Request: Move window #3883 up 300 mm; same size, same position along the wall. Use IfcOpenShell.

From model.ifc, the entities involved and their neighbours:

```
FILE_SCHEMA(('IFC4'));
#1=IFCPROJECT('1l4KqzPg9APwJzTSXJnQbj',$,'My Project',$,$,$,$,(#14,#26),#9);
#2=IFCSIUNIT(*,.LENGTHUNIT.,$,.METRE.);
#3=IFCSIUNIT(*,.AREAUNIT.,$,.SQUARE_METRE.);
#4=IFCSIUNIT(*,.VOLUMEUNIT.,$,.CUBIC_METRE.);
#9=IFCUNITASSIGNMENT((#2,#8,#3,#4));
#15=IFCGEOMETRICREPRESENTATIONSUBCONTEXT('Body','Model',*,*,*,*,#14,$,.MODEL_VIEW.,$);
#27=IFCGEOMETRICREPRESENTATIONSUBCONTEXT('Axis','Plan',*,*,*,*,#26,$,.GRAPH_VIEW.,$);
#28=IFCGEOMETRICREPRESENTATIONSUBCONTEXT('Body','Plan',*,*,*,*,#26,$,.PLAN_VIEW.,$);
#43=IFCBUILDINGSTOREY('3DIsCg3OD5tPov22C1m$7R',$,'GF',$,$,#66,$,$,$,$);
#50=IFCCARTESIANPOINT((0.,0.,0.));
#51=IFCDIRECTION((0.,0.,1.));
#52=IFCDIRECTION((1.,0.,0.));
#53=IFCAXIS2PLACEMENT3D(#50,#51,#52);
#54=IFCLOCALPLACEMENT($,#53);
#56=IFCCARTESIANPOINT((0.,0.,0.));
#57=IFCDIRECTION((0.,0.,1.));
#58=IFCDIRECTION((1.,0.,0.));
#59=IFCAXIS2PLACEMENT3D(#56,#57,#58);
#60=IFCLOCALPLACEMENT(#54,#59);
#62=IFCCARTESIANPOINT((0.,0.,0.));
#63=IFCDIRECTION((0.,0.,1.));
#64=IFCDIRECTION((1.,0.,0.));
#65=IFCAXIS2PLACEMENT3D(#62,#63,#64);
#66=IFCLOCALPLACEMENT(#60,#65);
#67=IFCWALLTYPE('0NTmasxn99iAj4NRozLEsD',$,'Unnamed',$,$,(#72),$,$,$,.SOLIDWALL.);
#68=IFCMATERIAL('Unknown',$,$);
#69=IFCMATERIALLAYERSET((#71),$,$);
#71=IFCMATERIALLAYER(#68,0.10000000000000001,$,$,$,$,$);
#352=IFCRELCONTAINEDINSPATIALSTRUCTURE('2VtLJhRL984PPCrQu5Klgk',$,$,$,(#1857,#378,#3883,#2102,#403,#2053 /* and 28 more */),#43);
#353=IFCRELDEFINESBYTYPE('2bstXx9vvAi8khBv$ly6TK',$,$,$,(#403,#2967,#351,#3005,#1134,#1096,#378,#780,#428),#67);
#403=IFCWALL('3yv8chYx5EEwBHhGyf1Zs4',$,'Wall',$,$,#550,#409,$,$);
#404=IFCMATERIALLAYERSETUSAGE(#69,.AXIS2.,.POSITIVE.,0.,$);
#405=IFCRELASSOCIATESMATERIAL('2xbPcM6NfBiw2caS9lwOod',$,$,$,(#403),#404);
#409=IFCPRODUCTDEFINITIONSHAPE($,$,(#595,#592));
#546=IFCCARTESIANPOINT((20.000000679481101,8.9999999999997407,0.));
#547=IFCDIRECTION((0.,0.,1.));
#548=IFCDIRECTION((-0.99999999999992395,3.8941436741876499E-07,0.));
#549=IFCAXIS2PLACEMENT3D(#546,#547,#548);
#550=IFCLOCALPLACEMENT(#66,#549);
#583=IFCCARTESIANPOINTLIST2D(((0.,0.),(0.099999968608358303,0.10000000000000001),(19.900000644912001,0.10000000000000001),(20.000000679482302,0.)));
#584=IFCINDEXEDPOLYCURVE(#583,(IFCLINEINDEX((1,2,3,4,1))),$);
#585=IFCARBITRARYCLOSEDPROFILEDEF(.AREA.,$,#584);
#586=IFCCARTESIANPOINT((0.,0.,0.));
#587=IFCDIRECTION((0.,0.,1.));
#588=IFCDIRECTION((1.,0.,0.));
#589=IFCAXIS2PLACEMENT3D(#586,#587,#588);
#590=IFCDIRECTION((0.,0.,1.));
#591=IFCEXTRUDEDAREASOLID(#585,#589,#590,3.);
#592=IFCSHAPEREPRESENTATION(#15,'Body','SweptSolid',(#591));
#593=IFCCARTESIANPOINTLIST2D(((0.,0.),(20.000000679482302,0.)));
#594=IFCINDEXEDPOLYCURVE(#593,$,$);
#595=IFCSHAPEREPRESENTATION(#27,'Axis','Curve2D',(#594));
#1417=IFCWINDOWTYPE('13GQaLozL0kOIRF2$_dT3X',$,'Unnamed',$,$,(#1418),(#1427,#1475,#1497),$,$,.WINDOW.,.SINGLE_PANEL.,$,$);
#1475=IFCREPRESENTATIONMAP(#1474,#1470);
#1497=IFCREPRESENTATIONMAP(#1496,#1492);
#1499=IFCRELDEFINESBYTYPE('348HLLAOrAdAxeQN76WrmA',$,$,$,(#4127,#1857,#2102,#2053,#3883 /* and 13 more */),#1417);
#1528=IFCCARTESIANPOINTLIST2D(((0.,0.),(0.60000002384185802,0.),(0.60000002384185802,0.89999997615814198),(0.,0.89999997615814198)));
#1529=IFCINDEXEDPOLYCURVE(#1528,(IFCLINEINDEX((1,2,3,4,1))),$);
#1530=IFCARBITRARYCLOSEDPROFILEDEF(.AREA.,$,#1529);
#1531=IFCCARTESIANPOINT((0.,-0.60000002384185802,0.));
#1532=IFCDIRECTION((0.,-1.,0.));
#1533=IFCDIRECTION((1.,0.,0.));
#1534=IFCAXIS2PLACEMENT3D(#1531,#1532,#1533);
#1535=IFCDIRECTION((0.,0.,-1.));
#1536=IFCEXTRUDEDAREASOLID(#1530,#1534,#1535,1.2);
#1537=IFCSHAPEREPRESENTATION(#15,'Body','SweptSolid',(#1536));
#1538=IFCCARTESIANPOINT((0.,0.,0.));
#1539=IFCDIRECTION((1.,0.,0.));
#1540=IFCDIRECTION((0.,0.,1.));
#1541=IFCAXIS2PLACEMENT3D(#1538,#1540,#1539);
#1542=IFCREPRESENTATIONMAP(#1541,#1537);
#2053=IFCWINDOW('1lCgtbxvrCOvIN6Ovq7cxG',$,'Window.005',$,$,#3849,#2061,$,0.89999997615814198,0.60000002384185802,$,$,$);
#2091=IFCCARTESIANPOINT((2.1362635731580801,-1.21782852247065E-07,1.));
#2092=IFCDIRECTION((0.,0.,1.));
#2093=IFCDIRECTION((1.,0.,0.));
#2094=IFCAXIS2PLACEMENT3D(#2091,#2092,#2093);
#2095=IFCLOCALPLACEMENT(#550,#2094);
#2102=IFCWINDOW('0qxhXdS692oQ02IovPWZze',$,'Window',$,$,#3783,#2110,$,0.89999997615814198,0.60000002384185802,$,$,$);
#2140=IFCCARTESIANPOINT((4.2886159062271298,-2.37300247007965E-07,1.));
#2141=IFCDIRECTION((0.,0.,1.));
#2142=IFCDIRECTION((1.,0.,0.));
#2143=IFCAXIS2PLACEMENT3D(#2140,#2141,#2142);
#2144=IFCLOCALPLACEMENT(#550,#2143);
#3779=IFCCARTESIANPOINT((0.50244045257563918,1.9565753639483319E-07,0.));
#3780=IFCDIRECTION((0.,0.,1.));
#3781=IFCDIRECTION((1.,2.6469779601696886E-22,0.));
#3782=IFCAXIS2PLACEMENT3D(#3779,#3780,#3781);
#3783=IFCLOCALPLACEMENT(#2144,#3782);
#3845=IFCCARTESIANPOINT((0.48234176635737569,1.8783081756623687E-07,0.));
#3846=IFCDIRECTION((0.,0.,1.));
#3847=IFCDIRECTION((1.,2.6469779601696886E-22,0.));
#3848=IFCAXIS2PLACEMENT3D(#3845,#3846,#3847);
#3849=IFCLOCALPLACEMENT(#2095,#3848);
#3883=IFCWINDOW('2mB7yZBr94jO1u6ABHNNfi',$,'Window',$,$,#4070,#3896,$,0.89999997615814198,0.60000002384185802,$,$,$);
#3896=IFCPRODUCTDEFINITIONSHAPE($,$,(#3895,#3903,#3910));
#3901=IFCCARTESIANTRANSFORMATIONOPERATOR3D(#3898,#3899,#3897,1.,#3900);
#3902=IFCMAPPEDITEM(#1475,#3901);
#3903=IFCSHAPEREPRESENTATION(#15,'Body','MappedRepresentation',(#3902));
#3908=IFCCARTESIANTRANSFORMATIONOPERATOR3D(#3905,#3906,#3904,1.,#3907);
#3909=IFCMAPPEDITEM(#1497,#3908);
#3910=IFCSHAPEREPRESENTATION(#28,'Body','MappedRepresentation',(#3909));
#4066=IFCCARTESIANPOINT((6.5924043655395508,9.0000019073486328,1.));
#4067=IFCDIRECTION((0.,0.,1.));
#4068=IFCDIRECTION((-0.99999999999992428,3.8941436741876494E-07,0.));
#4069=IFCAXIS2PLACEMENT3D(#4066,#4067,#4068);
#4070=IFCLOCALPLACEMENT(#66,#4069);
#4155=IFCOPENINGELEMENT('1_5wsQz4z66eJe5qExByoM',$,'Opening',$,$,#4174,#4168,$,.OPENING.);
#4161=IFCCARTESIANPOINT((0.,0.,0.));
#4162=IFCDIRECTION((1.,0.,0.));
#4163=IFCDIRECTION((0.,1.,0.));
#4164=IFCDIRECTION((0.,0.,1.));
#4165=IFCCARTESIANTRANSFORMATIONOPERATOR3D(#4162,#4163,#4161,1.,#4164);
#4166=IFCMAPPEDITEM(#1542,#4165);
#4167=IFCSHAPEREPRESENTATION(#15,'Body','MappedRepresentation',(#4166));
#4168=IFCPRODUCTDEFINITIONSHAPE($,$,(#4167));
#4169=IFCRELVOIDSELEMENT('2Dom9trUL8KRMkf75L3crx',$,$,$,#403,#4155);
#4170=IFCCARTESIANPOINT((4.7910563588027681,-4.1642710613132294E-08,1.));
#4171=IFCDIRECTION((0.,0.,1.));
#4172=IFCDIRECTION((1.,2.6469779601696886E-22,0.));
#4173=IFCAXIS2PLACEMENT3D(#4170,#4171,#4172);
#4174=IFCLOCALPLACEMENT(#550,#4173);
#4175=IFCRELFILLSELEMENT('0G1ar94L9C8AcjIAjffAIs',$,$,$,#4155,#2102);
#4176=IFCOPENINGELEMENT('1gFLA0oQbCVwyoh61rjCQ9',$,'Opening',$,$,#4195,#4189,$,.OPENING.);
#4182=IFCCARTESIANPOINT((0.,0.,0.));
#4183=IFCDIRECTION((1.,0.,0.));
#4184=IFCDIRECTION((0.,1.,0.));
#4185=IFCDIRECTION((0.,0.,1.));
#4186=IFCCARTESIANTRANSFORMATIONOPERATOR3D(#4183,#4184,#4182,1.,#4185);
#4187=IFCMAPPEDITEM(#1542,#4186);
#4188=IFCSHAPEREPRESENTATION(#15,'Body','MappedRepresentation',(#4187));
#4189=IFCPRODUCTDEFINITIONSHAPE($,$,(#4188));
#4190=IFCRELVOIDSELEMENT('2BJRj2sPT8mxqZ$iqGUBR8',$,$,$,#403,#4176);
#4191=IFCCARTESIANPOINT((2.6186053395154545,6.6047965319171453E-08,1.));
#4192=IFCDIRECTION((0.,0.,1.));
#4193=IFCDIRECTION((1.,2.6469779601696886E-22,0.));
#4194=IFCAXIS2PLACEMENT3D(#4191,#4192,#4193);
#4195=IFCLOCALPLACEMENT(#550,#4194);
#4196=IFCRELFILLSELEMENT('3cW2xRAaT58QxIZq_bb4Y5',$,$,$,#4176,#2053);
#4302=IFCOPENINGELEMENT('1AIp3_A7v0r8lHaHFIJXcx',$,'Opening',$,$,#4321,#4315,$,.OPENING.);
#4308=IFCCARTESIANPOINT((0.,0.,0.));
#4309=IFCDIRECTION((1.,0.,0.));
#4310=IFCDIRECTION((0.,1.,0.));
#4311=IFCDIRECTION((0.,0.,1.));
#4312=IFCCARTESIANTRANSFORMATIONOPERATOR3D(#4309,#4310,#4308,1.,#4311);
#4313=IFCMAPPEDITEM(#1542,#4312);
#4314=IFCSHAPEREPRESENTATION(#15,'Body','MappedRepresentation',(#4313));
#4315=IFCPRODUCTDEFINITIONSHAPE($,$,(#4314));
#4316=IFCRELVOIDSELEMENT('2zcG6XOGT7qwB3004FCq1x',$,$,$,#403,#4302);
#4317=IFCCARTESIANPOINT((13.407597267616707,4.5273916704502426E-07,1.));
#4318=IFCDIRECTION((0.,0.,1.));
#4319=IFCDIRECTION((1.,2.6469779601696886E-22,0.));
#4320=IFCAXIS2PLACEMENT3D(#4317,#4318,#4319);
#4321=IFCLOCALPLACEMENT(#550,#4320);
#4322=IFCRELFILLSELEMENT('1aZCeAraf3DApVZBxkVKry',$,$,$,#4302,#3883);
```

```python
import numpy as np
import ifcopenshell
import ifcopenshell.api.geometry
import ifcopenshell.util.placement
import ifcopenshell.util.unit

model = ifcopenshell.open("model.ifc")
unit_scale = ifcopenshell.util.unit.calculate_unit_scale(model)

window = model.by_id(3883)
opening = window.FillsVoids[0].RelatingOpeningElement
dz = 0.3 / unit_scale

shift = np.array([0.0, 0.0, dz])
# The window is not placed relative to its opening, so move both.
for product in (opening, window):
    matrix = ifcopenshell.util.placement.get_local_placement(product.ObjectPlacement)
    matrix[:3, 3] += shift
    ifcopenshell.api.geometry.edit_object_placement(model, product=product, matrix=matrix, is_si=False)

print(f"moved by {dz * unit_scale:+.3f} m")

model.write("model_updated.ifc")
```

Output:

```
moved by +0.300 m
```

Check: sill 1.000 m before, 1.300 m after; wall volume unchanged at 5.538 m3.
